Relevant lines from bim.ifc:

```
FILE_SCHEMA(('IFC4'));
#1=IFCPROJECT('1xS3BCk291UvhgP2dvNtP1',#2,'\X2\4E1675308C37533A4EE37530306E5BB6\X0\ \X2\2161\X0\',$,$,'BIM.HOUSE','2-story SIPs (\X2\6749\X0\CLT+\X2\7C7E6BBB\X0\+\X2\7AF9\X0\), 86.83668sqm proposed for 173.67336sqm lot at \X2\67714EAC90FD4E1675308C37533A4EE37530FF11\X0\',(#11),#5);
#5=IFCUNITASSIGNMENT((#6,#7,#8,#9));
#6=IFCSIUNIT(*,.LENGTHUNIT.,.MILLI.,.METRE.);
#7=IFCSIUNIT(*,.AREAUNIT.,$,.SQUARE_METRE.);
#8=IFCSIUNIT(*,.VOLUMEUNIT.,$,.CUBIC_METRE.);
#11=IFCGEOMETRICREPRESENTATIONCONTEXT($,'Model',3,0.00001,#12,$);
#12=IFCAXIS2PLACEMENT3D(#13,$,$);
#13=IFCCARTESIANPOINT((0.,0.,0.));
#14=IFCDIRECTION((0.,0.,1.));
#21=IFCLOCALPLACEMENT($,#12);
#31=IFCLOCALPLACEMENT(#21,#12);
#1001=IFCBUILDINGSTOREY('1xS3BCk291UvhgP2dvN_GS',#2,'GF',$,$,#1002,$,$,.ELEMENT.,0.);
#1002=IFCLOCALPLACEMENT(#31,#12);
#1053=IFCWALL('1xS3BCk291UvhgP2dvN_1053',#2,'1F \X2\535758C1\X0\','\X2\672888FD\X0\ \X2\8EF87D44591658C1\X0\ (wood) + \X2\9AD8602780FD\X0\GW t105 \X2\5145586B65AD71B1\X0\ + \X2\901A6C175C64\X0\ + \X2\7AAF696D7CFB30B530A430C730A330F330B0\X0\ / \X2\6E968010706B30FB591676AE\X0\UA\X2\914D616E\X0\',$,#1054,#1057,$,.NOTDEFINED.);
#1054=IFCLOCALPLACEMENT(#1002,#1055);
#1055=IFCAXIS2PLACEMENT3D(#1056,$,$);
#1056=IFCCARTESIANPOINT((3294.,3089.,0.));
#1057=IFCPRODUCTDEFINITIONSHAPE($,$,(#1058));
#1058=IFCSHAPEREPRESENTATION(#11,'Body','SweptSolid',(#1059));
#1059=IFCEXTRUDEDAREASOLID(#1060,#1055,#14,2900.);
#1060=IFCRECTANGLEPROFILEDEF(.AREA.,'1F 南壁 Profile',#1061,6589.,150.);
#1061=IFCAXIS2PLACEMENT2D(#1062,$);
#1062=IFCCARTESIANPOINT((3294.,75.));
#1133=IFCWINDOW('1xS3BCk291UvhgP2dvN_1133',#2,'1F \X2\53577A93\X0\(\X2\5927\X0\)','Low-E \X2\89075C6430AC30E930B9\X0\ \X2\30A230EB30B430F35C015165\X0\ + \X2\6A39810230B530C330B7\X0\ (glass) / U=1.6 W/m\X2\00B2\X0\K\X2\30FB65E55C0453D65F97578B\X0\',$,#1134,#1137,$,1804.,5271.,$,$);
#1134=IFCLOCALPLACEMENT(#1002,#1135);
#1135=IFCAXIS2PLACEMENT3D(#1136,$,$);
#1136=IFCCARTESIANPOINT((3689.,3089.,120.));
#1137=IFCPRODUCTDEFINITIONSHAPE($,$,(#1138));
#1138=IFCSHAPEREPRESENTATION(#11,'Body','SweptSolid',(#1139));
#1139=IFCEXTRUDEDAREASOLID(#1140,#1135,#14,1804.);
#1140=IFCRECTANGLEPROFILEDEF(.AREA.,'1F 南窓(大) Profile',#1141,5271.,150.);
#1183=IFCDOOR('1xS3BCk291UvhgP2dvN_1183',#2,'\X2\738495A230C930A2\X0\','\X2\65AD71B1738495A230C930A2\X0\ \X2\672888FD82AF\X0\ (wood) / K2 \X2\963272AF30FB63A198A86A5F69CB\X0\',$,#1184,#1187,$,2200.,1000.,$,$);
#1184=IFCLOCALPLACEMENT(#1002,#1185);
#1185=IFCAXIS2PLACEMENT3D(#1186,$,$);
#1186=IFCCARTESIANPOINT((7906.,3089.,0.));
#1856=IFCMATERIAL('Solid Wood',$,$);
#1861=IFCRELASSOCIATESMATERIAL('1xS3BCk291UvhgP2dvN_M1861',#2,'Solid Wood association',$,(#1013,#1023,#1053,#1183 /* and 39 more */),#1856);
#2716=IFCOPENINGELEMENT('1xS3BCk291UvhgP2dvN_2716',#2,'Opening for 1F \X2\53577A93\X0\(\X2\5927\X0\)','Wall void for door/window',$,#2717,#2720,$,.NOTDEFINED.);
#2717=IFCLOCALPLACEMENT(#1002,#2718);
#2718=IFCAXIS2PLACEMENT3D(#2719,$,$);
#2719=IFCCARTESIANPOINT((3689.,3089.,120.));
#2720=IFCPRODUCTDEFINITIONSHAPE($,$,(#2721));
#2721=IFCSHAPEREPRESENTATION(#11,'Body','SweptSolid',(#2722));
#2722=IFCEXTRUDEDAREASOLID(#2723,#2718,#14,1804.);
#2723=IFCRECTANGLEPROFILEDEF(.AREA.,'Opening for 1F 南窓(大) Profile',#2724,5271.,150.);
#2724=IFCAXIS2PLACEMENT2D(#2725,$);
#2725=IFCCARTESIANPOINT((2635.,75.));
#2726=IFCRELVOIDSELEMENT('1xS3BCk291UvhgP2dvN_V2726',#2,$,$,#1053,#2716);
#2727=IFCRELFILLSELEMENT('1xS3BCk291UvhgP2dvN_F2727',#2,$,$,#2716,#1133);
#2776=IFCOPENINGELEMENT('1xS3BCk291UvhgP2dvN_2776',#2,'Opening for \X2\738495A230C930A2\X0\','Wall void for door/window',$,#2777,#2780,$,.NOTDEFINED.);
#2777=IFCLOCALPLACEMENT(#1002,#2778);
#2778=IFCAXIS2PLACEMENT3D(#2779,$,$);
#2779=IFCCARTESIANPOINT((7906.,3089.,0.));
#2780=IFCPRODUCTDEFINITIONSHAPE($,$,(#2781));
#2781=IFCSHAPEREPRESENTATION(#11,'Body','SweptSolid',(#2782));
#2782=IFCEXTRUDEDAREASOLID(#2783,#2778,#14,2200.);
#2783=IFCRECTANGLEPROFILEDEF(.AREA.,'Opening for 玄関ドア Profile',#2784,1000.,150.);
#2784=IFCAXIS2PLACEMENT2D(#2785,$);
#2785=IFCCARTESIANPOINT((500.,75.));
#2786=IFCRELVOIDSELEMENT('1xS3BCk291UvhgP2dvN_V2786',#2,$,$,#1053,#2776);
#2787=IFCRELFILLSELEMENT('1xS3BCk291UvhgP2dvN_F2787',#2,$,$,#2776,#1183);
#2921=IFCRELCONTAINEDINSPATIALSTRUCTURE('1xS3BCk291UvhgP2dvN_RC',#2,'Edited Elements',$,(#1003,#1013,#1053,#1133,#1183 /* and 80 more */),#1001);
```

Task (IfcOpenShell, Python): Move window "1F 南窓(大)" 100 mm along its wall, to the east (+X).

```python
import ifcopenshell
import ifcopenshell.api.geometry
import ifcopenshell.util.placement

model = ifcopenshell.open("bim.ifc")

window = model.by_guid("1xS3BCk291UvhgP2dvN_1133")
opening = window.FillsVoids[0].RelatingOpeningElement
wall = opening.VoidsElements[0].RelatingBuildingElement

wall_matrix = ifcopenshell.util.placement.get_local_placement(wall.ObjectPlacement)
shift = wall_matrix[:3, 0] * 100.0
before = ifcopenshell.util.placement.get_local_placement(window.ObjectPlacement)[:3, 3].copy()

# The window is not placed relative to its opening, so move both.
for product in (opening, window):
    matrix = ifcopenshell.util.placement.get_local_placement(product.ObjectPlacement)
    matrix[:3, 3] += shift
    ifcopenshell.api.geometry.edit_object_placement(model, product=product, matrix=matrix, is_si=False)

after = ifcopenshell.util.placement.get_local_placement(window.ObjectPlacement)[:3, 3]
print("window moved by", (after - before).round(3) + 0.0)

model.write("bim_updated.ifc")
```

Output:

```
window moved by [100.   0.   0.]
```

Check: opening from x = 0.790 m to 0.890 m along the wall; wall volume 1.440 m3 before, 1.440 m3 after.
